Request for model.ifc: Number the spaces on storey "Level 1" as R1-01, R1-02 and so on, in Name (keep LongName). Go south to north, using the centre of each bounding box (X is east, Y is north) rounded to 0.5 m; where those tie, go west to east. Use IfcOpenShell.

First a look at what the model holds.

```python
import ifcopenshell
import ifcopenshell.util.element
import ifcopenshell.util.placement

model = ifcopenshell.open("model.ifc")
print(model.schema)
storey = next(s for s in model.by_type("IfcBuildingStorey") if s.Name == "Level 1")
spaces = [e for e in ifcopenshell.util.element.get_decomposition(storey) if e.is_a("IfcSpace")]
for e in sorted(spaces, key=lambda e: e.id()):
    origin = ifcopenshell.util.placement.get_local_placement(e.ObjectPlacement)[:3, 3]
    print(e.id(), e.Name, e.LongName, origin.round(2) + 0.0, sep=" | ")
```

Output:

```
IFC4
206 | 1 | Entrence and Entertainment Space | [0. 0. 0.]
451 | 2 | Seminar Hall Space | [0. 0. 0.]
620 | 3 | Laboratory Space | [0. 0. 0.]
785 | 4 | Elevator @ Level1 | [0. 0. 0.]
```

```python
import ifcopenshell
import ifcopenshell.geom
import ifcopenshell.util.element
import ifcopenshell.util.shape

model = ifcopenshell.open("model.ifc")
settings = ifcopenshell.geom.settings()
settings.set("use-world-coords", True)


def centre(element):
    shape = ifcopenshell.geom.create_shape(settings, element)
    return ifcopenshell.util.shape.get_bbox_centroid(shape.geometry)


storey = next(s for s in model.by_type("IfcBuildingStorey") if s.Name == "Level 1")
spaces = [e for e in ifcopenshell.util.element.get_decomposition(storey) if e.is_a("IfcSpace")]

# Insertion points can sit at a corner or the storey origin, so sort by the geometry (in metres).
centres = {e: centre(e) for e in spaces}
spaces.sort(key=lambda e: (round(centres[e][1] / 0.5), centres[e][0]))

for i, e in enumerate(spaces, start=1):
    number = f"R1-{i:02d}"
    e.Name = number
    print(e.id(), number)

model.write("model_rev.ifc")
```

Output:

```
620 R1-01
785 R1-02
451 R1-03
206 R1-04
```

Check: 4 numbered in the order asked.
